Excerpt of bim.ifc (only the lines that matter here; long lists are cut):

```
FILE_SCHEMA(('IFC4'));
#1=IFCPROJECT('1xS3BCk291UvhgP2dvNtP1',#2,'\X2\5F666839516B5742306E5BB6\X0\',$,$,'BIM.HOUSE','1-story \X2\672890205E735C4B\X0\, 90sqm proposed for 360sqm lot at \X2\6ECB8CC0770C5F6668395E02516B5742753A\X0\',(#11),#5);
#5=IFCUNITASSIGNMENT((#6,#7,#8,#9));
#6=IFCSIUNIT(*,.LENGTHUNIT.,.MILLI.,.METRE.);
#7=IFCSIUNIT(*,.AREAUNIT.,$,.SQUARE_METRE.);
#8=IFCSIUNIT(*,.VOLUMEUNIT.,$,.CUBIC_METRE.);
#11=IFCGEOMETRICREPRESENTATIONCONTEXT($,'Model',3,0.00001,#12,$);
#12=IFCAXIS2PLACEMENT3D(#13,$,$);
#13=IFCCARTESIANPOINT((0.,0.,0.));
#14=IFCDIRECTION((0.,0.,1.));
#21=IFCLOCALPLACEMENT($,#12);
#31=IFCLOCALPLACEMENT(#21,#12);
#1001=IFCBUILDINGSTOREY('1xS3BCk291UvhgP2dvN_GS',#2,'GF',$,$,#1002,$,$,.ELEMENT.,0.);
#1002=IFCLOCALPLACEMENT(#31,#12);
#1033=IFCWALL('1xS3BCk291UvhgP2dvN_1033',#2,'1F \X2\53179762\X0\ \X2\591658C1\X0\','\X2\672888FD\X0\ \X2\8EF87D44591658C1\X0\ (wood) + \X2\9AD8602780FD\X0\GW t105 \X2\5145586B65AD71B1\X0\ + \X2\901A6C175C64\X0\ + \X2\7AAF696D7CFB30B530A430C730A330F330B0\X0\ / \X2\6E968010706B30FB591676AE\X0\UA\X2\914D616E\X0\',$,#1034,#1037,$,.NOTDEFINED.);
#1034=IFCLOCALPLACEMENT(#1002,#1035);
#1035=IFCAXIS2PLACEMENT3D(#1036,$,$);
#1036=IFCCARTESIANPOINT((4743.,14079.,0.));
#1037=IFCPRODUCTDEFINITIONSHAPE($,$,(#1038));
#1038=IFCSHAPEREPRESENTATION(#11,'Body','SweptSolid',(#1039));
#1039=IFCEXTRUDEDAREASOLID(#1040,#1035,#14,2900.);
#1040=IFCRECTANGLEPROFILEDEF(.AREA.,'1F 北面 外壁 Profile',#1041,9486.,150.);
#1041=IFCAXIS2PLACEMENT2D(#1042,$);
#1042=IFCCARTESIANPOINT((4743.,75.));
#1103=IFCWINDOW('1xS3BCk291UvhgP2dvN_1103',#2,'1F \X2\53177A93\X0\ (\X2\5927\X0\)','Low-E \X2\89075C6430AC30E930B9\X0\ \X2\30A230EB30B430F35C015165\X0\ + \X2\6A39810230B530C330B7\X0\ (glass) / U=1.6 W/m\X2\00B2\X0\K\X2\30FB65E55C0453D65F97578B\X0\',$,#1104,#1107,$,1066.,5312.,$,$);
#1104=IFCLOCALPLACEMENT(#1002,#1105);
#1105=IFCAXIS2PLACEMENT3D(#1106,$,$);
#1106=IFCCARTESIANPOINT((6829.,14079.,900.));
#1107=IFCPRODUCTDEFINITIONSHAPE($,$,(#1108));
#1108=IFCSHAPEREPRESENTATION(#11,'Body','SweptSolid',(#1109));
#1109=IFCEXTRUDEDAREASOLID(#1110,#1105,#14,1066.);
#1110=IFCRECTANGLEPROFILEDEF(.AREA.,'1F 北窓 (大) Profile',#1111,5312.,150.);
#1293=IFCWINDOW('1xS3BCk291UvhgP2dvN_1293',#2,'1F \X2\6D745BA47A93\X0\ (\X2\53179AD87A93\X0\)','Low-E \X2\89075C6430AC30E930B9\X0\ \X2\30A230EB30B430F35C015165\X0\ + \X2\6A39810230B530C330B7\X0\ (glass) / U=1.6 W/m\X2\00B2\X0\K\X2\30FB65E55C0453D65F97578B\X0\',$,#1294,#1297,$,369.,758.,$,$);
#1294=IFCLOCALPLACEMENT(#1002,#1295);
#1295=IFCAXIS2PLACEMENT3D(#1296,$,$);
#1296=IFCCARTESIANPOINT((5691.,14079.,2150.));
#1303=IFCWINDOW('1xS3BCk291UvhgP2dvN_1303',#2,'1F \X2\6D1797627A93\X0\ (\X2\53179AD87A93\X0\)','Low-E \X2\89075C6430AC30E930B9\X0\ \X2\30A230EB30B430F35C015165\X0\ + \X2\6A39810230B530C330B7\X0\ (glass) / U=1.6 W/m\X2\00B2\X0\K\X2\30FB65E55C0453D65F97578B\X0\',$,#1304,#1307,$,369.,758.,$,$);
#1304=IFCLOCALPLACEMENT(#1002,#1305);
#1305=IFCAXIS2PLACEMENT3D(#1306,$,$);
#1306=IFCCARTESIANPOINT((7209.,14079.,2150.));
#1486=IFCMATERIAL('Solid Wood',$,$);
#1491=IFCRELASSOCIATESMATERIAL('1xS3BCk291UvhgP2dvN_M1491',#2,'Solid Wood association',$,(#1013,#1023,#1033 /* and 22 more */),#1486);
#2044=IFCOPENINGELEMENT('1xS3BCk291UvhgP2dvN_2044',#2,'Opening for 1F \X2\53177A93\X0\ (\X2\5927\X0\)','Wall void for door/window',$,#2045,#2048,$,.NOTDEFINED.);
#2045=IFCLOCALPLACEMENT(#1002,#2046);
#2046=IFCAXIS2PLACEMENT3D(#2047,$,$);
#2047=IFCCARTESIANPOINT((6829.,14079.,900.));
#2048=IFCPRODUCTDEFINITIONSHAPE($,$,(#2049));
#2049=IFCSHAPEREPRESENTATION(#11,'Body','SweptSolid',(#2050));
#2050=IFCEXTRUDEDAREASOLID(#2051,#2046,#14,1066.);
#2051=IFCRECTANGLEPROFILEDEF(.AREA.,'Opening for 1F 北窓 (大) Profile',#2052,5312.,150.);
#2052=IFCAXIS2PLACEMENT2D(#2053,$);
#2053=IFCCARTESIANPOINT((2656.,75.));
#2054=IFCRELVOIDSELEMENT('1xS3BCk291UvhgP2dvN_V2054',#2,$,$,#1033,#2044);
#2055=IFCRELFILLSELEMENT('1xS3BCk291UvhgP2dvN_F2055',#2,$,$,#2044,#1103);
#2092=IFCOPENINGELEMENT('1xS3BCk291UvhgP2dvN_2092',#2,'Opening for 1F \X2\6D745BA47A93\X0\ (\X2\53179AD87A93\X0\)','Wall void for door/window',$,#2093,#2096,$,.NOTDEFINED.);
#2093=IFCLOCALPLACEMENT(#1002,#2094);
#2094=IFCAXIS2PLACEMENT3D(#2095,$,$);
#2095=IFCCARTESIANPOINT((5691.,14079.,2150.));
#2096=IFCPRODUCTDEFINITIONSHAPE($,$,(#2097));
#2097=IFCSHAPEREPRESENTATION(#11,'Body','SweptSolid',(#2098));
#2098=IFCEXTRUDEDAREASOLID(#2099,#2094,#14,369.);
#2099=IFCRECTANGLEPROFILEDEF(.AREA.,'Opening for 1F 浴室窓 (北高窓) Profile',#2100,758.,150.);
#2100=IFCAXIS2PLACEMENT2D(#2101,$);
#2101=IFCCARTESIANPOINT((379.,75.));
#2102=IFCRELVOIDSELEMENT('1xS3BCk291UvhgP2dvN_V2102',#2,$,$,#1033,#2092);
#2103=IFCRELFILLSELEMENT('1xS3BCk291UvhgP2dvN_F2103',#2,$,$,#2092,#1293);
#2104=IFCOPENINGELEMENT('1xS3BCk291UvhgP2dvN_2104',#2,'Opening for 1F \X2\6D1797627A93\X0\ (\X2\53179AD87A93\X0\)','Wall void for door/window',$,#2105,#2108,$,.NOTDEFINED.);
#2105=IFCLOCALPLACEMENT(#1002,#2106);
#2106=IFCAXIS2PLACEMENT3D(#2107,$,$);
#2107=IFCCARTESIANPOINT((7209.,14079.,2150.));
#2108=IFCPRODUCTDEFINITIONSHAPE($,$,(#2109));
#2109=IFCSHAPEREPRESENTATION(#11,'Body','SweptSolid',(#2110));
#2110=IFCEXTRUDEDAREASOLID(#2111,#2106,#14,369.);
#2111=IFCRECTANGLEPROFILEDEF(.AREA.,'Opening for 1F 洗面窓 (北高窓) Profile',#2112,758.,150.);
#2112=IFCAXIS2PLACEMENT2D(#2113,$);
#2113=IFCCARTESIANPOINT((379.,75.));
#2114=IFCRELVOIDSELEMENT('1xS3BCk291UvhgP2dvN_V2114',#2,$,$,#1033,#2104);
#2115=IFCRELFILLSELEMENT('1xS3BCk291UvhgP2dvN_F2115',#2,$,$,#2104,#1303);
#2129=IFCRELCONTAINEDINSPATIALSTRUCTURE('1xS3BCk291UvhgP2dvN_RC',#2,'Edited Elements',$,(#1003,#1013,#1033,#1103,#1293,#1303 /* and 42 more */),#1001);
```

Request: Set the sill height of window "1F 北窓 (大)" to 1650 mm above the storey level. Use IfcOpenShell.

```python
import numpy as np
import ifcopenshell
import ifcopenshell.api.geometry
import ifcopenshell.geom
import ifcopenshell.util.element
import ifcopenshell.util.placement
import ifcopenshell.util.shape
import ifcopenshell.util.unit

model = ifcopenshell.open("bim.ifc")
unit_scale = ifcopenshell.util.unit.calculate_unit_scale(model)

window = model.by_guid("1xS3BCk291UvhgP2dvN_1103")
opening = window.FillsVoids[0].RelatingOpeningElement
storey = ifcopenshell.util.element.get_container(window, ifc_class="IfcBuildingStorey")
level = ifcopenshell.util.placement.get_local_placement(storey.ObjectPlacement)[2, 3]

# The opening's origin need not be at the sill, so measure its lowest point.
shape = ifcopenshell.geom.create_shape(ifcopenshell.geom.settings(), opening)
bottom = ifcopenshell.util.shape.get_shape_bottom_elevation(shape, shape.geometry) / unit_scale
dz = level + 1.65 / unit_scale - bottom

shift = np.array([0.0, 0.0, dz])
# The window is not placed relative to its opening, so move both.
for product in (opening, window):
    matrix = ifcopenshell.util.placement.get_local_placement(product.ObjectPlacement)
    matrix[:3, 3] += shift
    ifcopenshell.api.geometry.edit_object_placement(model, product=product, matrix=matrix, is_si=False)

print(f"moved by {dz * unit_scale:+.3f} m")

model.write("bim_rev.ifc")
```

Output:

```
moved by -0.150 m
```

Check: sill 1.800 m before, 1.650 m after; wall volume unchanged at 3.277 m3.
